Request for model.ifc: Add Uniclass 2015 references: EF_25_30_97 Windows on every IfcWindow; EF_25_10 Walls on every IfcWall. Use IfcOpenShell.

First a look at what the model holds.

```python
import ifcopenshell

model = ifcopenshell.open("model.ifc")
print(model.schema)
print("classifications:", [c.Name for c in model.by_type("IfcClassification")])
for ifc_class in ("IfcDoor", "IfcRoof", "IfcStair", "IfcWall", "IfcWindow"):
    print(ifc_class, len(model.by_type(ifc_class)))
```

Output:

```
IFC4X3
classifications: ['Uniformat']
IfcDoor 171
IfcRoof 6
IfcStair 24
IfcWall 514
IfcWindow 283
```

```python
import ifcopenshell
import ifcopenshell.api.classification

model = ifcopenshell.open("model.ifc")

system = ifcopenshell.api.classification.add_classification(model, classification="Uniclass 2015")

codes = {
    "IfcWindow": ("EF_25_30_97", "Windows"),
    "IfcWall": ("EF_25_10", "Walls"),
}
for ifc_class, (code, name) in codes.items():
    products = model.by_type(ifc_class)
    ifcopenshell.api.classification.add_reference(
        model, products=products, classification=system, identification=code, name=name
    )
    print(code, len(products))

model.write("model_updated.ifc")
```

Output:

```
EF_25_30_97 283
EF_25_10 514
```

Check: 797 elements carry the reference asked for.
